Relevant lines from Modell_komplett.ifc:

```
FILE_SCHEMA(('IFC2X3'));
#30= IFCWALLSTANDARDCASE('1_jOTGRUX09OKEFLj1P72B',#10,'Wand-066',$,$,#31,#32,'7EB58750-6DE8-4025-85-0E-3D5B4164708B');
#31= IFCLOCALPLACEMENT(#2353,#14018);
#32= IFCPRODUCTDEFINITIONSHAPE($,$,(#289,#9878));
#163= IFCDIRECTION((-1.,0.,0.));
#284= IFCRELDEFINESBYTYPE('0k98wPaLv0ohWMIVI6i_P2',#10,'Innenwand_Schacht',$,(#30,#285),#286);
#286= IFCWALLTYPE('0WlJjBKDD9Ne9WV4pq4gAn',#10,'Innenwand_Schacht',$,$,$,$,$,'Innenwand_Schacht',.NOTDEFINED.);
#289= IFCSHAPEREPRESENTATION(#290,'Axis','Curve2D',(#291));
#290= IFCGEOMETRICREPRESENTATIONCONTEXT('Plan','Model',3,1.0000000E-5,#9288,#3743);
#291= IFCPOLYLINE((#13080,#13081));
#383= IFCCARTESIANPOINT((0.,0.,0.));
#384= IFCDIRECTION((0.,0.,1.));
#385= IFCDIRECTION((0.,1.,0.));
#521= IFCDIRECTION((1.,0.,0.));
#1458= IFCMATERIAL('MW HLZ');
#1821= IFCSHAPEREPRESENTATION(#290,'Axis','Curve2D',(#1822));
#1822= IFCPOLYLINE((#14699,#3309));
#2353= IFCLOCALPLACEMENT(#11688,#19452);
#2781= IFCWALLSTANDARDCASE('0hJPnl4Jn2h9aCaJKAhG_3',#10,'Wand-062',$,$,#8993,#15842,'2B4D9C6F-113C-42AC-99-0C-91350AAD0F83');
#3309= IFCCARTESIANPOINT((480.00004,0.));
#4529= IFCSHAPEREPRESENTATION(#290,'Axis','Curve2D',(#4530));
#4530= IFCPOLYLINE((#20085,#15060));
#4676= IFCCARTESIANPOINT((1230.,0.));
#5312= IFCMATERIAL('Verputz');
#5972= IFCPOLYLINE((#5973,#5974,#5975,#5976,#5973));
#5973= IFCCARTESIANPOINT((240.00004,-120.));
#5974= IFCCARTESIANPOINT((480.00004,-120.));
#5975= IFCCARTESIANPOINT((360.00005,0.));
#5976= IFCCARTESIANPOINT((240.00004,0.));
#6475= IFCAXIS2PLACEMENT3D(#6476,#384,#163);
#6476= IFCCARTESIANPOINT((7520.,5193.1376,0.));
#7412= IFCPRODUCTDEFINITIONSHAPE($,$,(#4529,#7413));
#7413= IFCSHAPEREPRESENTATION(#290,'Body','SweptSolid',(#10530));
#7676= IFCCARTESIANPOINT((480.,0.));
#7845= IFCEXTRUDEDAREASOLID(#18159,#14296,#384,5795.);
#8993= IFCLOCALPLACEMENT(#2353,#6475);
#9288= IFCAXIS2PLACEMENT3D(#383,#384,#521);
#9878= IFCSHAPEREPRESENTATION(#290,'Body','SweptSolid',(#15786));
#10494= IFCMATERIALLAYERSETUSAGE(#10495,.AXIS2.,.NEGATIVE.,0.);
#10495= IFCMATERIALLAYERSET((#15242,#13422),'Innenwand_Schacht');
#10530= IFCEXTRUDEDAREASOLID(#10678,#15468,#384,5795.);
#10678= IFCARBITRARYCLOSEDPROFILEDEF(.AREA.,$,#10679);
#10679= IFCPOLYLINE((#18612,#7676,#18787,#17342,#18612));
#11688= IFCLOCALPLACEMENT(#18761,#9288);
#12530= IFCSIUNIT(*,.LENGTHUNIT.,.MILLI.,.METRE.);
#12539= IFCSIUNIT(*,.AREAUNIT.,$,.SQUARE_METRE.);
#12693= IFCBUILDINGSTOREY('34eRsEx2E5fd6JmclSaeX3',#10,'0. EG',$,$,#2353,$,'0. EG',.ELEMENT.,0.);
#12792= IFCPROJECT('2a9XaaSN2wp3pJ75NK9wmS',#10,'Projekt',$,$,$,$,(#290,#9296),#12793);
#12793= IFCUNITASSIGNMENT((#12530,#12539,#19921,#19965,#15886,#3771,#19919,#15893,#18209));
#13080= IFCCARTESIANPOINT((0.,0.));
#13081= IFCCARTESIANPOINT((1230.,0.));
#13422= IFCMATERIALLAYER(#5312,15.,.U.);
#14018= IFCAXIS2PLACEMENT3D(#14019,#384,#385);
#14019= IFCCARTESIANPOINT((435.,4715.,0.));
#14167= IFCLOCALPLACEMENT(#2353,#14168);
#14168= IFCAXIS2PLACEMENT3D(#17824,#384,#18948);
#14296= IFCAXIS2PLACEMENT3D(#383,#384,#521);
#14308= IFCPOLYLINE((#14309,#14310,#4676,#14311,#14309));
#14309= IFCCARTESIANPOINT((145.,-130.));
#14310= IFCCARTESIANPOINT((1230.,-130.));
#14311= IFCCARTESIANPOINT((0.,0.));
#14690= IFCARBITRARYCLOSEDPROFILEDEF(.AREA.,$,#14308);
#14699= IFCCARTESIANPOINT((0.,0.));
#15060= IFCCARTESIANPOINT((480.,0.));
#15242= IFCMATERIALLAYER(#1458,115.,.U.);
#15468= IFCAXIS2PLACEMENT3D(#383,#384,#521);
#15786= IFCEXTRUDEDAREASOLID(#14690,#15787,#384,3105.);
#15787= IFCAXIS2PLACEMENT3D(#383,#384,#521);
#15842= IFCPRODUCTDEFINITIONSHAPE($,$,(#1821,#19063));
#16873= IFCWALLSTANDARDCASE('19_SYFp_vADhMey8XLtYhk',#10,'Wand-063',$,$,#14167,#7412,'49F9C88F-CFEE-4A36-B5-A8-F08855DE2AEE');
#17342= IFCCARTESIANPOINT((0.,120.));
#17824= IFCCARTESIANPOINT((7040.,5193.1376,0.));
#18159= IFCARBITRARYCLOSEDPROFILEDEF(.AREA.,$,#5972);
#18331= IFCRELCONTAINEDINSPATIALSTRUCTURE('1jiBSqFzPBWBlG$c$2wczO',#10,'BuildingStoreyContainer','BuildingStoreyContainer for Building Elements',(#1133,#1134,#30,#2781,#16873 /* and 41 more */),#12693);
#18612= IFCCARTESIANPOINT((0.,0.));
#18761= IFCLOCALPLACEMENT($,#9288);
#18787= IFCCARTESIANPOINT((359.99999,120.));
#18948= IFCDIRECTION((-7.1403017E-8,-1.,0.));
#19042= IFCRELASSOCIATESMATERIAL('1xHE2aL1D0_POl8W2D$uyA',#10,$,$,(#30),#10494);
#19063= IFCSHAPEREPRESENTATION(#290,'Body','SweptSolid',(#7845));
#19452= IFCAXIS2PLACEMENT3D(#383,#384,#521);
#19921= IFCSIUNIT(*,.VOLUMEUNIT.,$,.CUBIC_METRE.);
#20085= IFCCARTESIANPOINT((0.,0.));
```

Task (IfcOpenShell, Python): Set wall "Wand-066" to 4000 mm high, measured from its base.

```python
import ifcopenshell
import ifcopenshell.geom
import ifcopenshell.util.shape
import ifcopenshell.util.unit

model = ifcopenshell.open("Modell_komplett.ifc")
unit_scale = ifcopenshell.util.unit.calculate_unit_scale(model)
settings = ifcopenshell.geom.settings()


def volume(element):
    """Net volume in cubic metres, openings subtracted."""
    shape = ifcopenshell.geom.create_shape(settings, element)
    return ifcopenshell.util.shape.get_volume(shape.geometry)


wall = model.by_guid("1_jOTGRUX09OKEFLj1P72B")
before = volume(wall)

body = next(r for r in wall.Representation.Representations if r.RepresentationIdentifier == "Body")
solid = body.Items[0]
old_height = solid.Depth
solid.Depth = 4 / unit_scale
after = volume(wall)

print(f"height {old_height:g} -> {solid.Depth:g}, volume {before:.3f} -> {after:.3f} m3")

model.write("Modell_komplett_v2.ifc")
```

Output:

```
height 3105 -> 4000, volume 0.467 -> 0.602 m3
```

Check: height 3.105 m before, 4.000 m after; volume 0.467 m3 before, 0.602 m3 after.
